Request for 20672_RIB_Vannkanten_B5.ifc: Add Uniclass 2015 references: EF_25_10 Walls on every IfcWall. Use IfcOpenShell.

First a look at what the model holds.

```python
import ifcopenshell

model = ifcopenshell.open("20672_RIB_Vannkanten_B5.ifc")
print(model.schema)
print("classifications:", [c.Name for c in model.by_type("IfcClassification")])
for ifc_class in ("IfcDoor", "IfcRoof", "IfcStair", "IfcWall", "IfcWindow"):
    print(ifc_class, len(model.by_type(ifc_class)))
```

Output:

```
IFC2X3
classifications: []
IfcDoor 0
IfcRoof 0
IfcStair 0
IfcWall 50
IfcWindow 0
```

```python
import ifcopenshell
import ifcopenshell.api.classification

model = ifcopenshell.open("20672_RIB_Vannkanten_B5.ifc")

# IFC2X3 requires Source and Edition and has no link from the project to the system.
system = model.create_entity("IfcClassification", Source="NBS", Edition="2015", Name="Uniclass 2015")

codes = {
    "IfcWall": ("EF_25_10", "Walls"),
}
for ifc_class, (code, name) in codes.items():
    products = model.by_type(ifc_class)
    ifcopenshell.api.classification.add_reference(
        model, products=products, classification=system, identification=code, name=name
    )
    print(code, len(products))

model.write("20672_RIB_Vannkanten_B5_updated.ifc")
```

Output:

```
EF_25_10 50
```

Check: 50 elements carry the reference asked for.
